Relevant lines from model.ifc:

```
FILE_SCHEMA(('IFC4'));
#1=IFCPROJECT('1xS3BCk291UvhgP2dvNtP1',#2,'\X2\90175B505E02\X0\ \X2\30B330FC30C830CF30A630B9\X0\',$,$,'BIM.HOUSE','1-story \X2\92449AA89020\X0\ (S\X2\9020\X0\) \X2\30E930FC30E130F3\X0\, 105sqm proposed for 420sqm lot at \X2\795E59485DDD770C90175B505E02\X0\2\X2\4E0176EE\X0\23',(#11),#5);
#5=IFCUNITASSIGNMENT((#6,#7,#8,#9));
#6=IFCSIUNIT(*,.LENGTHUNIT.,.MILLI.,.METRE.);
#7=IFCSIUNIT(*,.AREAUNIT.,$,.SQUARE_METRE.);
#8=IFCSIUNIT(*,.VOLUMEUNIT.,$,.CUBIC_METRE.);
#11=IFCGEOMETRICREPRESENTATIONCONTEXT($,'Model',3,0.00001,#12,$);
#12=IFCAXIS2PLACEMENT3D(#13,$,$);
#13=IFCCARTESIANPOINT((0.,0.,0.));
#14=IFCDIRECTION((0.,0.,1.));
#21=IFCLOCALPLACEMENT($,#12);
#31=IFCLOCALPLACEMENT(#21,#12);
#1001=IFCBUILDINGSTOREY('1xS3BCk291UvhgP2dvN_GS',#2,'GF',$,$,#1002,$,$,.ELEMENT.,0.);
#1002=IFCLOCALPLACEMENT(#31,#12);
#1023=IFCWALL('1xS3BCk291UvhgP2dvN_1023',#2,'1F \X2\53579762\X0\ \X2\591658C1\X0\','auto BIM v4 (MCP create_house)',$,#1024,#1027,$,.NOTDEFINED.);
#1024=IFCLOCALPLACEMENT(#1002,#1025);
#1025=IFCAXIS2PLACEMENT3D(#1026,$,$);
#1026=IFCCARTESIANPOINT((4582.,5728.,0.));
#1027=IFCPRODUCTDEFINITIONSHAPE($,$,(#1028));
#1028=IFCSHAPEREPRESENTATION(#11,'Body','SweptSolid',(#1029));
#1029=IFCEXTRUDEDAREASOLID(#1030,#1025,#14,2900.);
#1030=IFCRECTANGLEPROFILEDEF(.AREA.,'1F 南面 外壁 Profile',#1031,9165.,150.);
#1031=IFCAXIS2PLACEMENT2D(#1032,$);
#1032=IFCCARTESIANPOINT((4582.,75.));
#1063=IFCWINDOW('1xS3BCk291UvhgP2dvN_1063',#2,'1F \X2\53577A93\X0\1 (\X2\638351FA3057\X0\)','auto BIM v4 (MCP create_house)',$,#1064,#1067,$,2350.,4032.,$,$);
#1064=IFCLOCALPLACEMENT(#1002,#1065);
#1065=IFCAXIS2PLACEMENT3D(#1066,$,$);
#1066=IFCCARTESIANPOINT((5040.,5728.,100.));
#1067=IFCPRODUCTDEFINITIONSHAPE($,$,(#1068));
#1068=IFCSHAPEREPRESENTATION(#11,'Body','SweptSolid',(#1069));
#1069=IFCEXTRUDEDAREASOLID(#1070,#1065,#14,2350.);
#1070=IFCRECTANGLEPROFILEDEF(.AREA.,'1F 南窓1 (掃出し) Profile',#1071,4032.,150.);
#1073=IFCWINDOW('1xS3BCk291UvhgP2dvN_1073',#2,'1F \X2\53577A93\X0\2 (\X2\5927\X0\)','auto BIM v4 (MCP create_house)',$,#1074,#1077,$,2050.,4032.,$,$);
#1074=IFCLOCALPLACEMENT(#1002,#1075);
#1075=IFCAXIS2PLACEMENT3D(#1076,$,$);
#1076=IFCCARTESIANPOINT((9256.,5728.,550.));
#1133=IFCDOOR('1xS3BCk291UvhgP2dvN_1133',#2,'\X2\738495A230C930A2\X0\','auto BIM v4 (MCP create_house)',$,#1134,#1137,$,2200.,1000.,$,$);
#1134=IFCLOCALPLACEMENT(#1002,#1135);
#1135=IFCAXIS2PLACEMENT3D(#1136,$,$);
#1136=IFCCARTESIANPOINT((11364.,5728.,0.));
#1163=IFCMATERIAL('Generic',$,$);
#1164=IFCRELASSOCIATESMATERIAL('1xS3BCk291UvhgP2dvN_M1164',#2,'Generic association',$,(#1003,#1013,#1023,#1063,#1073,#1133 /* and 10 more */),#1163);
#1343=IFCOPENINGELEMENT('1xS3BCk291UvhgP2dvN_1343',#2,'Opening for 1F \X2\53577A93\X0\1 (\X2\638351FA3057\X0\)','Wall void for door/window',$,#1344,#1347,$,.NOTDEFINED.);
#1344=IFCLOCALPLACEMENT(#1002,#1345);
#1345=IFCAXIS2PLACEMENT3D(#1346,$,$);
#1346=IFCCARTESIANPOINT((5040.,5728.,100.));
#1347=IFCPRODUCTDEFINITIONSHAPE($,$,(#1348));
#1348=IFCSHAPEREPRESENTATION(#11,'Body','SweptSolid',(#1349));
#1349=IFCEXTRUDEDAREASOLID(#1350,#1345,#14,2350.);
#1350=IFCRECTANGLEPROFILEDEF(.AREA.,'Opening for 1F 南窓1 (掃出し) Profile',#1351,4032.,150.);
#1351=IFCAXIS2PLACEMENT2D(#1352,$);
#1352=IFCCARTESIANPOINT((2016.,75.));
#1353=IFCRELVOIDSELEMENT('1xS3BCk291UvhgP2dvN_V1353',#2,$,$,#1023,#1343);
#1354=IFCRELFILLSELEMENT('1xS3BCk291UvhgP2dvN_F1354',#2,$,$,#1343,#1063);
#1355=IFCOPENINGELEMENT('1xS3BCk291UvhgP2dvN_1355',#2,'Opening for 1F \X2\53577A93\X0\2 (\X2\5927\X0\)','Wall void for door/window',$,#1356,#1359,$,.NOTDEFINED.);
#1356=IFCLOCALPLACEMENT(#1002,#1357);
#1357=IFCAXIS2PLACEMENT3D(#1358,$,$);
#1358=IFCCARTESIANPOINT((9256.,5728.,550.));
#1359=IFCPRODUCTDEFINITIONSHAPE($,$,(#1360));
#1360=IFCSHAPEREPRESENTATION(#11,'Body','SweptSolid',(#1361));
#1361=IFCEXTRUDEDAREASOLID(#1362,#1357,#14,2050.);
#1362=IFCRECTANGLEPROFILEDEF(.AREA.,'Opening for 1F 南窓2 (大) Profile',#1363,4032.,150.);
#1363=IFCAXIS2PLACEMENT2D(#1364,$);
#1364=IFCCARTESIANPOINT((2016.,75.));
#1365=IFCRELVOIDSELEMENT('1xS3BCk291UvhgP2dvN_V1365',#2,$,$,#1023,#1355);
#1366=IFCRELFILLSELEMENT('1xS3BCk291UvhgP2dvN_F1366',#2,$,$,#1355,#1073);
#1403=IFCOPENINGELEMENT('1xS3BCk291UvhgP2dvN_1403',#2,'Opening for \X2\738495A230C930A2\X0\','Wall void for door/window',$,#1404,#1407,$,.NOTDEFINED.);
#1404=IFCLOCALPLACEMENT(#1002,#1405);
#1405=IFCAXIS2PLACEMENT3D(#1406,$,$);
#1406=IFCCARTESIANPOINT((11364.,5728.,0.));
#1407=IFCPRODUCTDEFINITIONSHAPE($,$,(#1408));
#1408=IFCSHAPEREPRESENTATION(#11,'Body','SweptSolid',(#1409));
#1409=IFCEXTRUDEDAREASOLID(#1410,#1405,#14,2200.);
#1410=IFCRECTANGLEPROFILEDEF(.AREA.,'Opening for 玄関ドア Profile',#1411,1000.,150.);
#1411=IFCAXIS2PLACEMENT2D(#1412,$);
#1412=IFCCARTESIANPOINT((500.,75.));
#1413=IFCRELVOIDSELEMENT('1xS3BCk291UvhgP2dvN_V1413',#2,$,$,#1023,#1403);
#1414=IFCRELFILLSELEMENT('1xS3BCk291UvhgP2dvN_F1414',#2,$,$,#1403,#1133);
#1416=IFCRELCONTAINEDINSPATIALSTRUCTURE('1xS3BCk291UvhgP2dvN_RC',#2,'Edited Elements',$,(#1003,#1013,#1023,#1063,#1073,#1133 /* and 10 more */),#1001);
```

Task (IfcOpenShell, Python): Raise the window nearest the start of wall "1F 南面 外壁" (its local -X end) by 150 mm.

```python
import numpy as np
import ifcopenshell
import ifcopenshell.api.geometry
import ifcopenshell.util.placement
import ifcopenshell.util.unit

model = ifcopenshell.open("model.ifc")
unit_scale = ifcopenshell.util.unit.calculate_unit_scale(model)

window = model.by_guid("1xS3BCk291UvhgP2dvN_1063")
opening = window.FillsVoids[0].RelatingOpeningElement
dz = 150.0

shift = np.array([0.0, 0.0, dz])
# The window is not placed relative to its opening, so move both.
for product in (opening, window):
    matrix = ifcopenshell.util.placement.get_local_placement(product.ObjectPlacement)
    matrix[:3, 3] += shift
    ifcopenshell.api.geometry.edit_object_placement(model, product=product, matrix=matrix, is_si=False)

print(f"moved by {dz * unit_scale:+.3f} m")

model.write("model_v2.ifc")
```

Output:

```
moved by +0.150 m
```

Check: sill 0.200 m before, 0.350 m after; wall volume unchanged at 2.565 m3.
